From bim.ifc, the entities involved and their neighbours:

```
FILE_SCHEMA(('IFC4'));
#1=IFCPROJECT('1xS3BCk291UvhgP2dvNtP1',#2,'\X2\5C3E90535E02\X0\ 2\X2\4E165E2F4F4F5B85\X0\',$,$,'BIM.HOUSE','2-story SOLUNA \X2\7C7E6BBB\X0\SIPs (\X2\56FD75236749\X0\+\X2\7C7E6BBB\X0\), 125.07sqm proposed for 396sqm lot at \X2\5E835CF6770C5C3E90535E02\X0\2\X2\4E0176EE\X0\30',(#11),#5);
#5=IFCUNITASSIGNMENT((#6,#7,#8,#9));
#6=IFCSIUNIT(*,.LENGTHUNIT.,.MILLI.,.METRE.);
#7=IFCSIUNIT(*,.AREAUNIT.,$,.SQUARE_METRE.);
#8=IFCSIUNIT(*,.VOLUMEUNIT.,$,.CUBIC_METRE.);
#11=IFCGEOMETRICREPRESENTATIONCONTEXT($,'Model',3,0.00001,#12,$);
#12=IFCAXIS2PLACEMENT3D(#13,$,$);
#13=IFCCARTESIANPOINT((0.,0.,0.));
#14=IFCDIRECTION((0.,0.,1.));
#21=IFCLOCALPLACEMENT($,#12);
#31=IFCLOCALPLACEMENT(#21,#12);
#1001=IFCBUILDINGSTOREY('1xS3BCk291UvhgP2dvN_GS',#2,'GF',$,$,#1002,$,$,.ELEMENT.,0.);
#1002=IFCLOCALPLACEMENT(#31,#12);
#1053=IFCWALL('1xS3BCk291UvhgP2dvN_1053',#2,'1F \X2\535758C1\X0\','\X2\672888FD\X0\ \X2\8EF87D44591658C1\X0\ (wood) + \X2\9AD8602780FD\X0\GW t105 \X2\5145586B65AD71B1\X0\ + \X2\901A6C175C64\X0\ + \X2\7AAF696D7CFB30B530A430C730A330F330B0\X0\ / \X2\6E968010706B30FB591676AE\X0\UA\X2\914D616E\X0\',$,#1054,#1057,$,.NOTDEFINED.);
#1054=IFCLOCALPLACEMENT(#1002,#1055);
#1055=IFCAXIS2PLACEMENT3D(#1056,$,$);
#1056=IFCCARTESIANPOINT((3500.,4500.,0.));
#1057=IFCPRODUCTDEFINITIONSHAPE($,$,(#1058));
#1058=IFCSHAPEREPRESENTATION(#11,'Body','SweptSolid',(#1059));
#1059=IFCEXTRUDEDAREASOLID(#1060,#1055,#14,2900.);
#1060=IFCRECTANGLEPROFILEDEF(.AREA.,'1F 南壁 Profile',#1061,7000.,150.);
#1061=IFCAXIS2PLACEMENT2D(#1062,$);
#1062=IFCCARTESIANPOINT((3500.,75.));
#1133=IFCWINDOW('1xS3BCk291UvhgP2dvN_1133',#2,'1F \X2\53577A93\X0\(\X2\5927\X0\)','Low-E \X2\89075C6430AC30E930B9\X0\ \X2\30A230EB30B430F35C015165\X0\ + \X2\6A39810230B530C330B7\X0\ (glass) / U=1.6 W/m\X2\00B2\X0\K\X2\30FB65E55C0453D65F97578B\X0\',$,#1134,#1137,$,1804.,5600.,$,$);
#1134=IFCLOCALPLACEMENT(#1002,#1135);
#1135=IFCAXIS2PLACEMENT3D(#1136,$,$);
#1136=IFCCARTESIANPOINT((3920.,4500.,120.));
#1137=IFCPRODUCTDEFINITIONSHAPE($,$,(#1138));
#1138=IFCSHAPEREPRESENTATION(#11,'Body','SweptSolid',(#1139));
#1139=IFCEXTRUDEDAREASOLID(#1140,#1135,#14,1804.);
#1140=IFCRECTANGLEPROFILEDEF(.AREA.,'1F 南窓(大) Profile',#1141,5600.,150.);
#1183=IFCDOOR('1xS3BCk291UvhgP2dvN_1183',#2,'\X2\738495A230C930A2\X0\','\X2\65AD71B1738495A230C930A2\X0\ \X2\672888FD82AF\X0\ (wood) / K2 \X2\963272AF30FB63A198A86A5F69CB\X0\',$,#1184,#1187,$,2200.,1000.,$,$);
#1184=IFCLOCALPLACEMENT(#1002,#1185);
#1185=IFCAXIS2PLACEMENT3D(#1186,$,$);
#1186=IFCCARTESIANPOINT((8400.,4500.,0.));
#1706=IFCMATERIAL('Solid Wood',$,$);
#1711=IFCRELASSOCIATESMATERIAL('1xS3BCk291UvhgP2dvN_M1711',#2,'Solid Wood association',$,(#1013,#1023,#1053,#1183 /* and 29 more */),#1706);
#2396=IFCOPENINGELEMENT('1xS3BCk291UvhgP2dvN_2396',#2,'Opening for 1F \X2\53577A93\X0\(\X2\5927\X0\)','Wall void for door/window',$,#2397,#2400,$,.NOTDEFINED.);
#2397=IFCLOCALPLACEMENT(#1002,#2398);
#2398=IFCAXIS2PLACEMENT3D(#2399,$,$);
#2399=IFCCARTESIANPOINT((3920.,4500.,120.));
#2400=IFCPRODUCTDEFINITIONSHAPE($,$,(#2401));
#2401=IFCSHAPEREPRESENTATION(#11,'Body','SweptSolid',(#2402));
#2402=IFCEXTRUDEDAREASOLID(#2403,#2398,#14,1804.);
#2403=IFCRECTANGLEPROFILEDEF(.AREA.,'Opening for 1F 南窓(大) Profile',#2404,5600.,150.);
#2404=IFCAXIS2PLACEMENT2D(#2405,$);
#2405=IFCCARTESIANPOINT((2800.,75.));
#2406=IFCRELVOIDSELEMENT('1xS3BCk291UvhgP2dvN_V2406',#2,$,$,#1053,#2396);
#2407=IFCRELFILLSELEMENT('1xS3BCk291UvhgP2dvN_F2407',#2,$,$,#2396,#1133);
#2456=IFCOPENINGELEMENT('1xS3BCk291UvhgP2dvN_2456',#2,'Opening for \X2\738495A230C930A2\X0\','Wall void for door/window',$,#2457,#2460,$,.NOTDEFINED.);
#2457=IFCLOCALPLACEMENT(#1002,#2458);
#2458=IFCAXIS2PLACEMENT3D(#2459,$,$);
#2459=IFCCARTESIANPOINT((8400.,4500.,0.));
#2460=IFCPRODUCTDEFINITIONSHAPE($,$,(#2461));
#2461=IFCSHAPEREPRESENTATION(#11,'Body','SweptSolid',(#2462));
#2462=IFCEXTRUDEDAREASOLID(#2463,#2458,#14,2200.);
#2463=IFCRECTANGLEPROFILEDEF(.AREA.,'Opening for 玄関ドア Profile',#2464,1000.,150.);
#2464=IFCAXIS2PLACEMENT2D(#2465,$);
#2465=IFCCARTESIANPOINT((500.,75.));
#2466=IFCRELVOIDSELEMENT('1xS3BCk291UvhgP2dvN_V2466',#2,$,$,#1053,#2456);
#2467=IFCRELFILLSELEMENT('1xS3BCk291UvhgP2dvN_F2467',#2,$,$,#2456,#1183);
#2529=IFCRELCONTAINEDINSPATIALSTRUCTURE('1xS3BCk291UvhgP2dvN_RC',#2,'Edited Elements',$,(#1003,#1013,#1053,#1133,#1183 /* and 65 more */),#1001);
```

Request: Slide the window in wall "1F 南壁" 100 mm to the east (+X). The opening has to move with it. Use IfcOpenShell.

```python
import ifcopenshell
import ifcopenshell.api.geometry
import ifcopenshell.util.placement
import ifcopenshell.util.unit

model = ifcopenshell.open("bim.ifc")
unit_scale = ifcopenshell.util.unit.calculate_unit_scale(model)

window = model.by_guid("1xS3BCk291UvhgP2dvN_1133")
opening = window.FillsVoids[0].RelatingOpeningElement
wall = opening.VoidsElements[0].RelatingBuildingElement

wall_matrix = ifcopenshell.util.placement.get_local_placement(wall.ObjectPlacement)
shift = wall_matrix[:3, 0] * 0.1 / unit_scale
before = ifcopenshell.util.placement.get_local_placement(window.ObjectPlacement)[:3, 3].copy()

# The window is not placed relative to its opening, so move both.
for product in (opening, window):
    matrix = ifcopenshell.util.placement.get_local_placement(product.ObjectPlacement)
    matrix[:3, 3] += shift
    ifcopenshell.api.geometry.edit_object_placement(model, product=product, matrix=matrix, is_si=False)

after = ifcopenshell.util.placement.get_local_placement(window.ObjectPlacement)[:3, 3]
print("window moved by", (after - before).round(3) + 0.0)

model.write("bim_rev.ifc")
```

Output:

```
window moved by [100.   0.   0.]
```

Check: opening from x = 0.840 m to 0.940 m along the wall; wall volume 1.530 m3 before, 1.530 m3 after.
